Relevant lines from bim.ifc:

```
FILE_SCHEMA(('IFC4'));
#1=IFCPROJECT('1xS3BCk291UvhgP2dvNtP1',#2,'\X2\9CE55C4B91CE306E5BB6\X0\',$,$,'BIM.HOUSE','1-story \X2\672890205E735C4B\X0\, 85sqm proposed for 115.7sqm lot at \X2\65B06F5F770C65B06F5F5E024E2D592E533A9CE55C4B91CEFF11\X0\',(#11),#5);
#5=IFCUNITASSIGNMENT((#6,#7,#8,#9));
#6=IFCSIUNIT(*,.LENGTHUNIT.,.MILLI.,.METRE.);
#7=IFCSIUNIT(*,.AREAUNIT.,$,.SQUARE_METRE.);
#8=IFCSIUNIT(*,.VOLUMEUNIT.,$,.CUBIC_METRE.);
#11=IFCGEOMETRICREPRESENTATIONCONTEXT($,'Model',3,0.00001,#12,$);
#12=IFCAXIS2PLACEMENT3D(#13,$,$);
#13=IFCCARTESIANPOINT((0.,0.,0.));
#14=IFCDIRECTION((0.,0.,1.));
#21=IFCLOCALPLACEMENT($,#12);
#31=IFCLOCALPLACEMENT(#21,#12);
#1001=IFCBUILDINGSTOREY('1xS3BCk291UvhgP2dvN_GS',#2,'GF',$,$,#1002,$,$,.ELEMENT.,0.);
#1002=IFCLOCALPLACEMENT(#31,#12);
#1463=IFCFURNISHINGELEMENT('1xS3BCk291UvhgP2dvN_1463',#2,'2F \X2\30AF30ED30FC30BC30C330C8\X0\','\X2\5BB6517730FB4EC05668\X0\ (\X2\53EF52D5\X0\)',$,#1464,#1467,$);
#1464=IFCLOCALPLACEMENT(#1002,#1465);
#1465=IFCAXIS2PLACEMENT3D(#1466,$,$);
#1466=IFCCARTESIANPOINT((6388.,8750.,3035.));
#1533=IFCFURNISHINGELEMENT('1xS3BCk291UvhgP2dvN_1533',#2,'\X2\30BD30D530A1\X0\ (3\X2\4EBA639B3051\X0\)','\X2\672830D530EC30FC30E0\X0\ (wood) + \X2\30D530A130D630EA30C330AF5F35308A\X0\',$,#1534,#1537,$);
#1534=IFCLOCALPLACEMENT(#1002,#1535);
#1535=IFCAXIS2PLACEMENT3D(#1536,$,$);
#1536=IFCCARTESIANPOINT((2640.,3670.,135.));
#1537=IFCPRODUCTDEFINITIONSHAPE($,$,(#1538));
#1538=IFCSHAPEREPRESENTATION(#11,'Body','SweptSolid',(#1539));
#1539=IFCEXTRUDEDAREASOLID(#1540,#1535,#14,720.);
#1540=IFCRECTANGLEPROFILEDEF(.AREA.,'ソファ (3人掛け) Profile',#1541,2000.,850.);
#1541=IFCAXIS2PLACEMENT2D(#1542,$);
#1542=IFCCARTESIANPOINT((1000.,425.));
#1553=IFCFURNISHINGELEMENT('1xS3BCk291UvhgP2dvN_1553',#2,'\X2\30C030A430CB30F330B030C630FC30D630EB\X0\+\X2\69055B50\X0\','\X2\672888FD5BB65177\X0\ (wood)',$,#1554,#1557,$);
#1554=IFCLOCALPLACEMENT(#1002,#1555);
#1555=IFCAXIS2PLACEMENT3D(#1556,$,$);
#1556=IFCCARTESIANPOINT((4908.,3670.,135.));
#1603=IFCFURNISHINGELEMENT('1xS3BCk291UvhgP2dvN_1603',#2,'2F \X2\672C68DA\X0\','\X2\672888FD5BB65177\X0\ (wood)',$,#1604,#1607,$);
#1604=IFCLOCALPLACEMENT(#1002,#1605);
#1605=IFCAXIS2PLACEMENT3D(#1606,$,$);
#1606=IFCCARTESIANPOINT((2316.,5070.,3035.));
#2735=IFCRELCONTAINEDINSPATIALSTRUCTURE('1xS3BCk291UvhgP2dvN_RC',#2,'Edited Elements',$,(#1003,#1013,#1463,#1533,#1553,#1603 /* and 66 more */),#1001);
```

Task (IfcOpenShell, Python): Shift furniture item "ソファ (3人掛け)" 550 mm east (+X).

```python
import ifcopenshell
import ifcopenshell.api.geometry
import ifcopenshell.util.placement

model = ifcopenshell.open("bim.ifc")

item = model.by_guid("1xS3BCk291UvhgP2dvN_1533")
matrix = ifcopenshell.util.placement.get_local_placement(item.ObjectPlacement)
matrix[0, 3] += 550.0
ifcopenshell.api.geometry.edit_object_placement(model, product=item, matrix=matrix, is_si=False)

print(ifcopenshell.util.placement.get_local_placement(item.ObjectPlacement).round(3) + 0.0)

model.write("bim_rev.ifc")
```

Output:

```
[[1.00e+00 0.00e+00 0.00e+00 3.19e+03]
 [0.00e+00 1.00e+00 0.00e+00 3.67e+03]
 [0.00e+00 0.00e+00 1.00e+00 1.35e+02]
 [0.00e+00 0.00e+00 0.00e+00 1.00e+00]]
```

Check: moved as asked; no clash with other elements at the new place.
